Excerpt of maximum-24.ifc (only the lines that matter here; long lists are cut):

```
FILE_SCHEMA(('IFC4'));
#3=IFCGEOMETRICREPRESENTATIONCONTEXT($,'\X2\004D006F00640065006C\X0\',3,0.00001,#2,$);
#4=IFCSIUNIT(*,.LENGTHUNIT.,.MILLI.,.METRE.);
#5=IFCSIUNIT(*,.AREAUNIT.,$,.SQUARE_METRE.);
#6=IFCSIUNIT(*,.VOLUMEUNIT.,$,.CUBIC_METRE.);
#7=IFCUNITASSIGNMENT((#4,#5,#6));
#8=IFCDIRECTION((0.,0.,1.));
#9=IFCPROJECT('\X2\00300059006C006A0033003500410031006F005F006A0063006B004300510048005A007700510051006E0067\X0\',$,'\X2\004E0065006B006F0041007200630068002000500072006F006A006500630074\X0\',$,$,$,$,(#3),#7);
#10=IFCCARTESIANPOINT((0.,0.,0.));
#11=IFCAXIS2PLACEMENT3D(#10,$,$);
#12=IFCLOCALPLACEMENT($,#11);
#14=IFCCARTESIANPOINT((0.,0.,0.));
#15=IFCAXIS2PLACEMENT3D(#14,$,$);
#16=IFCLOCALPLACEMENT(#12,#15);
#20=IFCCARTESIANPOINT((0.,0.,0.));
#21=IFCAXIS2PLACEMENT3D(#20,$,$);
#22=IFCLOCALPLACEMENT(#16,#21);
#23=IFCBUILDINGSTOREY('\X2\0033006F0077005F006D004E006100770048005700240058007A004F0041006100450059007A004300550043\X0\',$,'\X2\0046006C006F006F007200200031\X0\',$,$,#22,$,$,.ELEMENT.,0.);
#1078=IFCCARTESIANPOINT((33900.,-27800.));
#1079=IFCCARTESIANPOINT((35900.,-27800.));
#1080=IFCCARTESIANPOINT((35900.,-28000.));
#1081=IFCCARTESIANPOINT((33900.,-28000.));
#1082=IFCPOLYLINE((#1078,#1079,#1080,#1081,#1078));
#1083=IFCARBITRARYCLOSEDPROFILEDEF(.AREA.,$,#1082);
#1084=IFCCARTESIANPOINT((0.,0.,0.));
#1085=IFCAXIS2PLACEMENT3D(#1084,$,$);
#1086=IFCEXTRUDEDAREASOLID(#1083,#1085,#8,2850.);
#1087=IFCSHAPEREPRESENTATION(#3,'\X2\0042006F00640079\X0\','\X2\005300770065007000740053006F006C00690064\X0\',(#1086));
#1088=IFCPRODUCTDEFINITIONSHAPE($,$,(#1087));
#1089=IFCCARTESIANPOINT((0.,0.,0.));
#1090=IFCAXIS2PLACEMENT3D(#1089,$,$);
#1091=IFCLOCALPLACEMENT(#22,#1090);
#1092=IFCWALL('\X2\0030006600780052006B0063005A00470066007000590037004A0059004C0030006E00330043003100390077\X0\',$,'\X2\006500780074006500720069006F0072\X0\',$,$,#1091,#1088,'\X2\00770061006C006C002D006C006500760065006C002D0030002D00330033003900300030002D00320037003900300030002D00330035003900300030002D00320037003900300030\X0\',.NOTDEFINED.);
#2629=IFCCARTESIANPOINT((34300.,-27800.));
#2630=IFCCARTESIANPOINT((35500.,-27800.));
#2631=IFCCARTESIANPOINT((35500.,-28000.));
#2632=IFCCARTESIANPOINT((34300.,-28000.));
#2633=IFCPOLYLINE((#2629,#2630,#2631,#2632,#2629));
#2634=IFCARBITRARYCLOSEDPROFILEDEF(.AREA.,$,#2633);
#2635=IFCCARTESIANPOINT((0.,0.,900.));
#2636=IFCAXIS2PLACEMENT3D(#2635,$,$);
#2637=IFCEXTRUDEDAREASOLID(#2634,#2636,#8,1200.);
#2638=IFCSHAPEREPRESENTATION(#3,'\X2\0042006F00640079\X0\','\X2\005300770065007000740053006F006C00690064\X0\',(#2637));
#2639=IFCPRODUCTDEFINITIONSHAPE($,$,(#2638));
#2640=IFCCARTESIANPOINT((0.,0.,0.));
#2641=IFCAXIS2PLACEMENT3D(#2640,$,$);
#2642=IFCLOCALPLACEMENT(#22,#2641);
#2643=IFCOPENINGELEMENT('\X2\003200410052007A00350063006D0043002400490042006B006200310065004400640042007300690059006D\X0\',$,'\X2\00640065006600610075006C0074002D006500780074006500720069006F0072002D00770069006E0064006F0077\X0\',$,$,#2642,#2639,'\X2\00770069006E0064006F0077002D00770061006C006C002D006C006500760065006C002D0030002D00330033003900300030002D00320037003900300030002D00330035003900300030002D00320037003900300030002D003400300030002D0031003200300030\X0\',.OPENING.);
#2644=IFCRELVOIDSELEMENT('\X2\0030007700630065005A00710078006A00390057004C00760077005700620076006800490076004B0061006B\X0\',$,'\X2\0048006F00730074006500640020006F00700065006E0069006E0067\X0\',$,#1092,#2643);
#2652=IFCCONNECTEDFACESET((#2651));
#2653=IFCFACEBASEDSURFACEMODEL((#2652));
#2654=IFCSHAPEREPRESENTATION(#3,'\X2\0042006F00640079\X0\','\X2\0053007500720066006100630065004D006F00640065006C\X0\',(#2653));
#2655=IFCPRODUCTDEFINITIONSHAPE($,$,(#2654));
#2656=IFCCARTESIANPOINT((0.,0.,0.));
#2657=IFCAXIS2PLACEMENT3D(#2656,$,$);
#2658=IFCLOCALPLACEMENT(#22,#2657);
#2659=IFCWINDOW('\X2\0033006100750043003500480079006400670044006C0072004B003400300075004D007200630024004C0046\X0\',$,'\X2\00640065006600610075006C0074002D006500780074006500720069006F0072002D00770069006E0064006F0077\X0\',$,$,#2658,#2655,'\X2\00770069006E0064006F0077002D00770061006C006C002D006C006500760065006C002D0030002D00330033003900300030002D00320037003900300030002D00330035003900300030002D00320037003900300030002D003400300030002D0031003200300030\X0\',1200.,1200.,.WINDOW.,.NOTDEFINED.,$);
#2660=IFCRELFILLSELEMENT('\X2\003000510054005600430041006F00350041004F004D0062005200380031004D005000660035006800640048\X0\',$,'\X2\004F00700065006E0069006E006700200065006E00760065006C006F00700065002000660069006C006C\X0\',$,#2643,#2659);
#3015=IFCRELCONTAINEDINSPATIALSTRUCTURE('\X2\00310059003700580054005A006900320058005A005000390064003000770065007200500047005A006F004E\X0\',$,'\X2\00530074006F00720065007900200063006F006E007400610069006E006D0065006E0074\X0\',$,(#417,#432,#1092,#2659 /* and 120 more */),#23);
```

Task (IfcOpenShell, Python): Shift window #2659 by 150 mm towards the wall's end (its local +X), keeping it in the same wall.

```python
import ifcopenshell
import ifcopenshell.api.geometry
import ifcopenshell.util.placement
import ifcopenshell.util.unit

model = ifcopenshell.open("maximum-24.ifc")
unit_scale = ifcopenshell.util.unit.calculate_unit_scale(model)

window = model.by_id(2659)
opening = window.FillsVoids[0].RelatingOpeningElement
wall = opening.VoidsElements[0].RelatingBuildingElement

wall_matrix = ifcopenshell.util.placement.get_local_placement(wall.ObjectPlacement)
shift = wall_matrix[:3, 0] * 0.15 / unit_scale
before = ifcopenshell.util.placement.get_local_placement(window.ObjectPlacement)[:3, 3].copy()

# The window is not placed relative to its opening, so move both.
for product in (opening, window):
    matrix = ifcopenshell.util.placement.get_local_placement(product.ObjectPlacement)
    matrix[:3, 3] += shift
    ifcopenshell.api.geometry.edit_object_placement(model, product=product, matrix=matrix, is_si=False)

after = ifcopenshell.util.placement.get_local_placement(window.ObjectPlacement)[:3, 3]
print("window moved by", (after - before).round(3) + 0.0)

model.write("maximum-24_v2.ifc")
```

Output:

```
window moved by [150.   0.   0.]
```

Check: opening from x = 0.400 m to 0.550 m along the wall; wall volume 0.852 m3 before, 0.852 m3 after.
